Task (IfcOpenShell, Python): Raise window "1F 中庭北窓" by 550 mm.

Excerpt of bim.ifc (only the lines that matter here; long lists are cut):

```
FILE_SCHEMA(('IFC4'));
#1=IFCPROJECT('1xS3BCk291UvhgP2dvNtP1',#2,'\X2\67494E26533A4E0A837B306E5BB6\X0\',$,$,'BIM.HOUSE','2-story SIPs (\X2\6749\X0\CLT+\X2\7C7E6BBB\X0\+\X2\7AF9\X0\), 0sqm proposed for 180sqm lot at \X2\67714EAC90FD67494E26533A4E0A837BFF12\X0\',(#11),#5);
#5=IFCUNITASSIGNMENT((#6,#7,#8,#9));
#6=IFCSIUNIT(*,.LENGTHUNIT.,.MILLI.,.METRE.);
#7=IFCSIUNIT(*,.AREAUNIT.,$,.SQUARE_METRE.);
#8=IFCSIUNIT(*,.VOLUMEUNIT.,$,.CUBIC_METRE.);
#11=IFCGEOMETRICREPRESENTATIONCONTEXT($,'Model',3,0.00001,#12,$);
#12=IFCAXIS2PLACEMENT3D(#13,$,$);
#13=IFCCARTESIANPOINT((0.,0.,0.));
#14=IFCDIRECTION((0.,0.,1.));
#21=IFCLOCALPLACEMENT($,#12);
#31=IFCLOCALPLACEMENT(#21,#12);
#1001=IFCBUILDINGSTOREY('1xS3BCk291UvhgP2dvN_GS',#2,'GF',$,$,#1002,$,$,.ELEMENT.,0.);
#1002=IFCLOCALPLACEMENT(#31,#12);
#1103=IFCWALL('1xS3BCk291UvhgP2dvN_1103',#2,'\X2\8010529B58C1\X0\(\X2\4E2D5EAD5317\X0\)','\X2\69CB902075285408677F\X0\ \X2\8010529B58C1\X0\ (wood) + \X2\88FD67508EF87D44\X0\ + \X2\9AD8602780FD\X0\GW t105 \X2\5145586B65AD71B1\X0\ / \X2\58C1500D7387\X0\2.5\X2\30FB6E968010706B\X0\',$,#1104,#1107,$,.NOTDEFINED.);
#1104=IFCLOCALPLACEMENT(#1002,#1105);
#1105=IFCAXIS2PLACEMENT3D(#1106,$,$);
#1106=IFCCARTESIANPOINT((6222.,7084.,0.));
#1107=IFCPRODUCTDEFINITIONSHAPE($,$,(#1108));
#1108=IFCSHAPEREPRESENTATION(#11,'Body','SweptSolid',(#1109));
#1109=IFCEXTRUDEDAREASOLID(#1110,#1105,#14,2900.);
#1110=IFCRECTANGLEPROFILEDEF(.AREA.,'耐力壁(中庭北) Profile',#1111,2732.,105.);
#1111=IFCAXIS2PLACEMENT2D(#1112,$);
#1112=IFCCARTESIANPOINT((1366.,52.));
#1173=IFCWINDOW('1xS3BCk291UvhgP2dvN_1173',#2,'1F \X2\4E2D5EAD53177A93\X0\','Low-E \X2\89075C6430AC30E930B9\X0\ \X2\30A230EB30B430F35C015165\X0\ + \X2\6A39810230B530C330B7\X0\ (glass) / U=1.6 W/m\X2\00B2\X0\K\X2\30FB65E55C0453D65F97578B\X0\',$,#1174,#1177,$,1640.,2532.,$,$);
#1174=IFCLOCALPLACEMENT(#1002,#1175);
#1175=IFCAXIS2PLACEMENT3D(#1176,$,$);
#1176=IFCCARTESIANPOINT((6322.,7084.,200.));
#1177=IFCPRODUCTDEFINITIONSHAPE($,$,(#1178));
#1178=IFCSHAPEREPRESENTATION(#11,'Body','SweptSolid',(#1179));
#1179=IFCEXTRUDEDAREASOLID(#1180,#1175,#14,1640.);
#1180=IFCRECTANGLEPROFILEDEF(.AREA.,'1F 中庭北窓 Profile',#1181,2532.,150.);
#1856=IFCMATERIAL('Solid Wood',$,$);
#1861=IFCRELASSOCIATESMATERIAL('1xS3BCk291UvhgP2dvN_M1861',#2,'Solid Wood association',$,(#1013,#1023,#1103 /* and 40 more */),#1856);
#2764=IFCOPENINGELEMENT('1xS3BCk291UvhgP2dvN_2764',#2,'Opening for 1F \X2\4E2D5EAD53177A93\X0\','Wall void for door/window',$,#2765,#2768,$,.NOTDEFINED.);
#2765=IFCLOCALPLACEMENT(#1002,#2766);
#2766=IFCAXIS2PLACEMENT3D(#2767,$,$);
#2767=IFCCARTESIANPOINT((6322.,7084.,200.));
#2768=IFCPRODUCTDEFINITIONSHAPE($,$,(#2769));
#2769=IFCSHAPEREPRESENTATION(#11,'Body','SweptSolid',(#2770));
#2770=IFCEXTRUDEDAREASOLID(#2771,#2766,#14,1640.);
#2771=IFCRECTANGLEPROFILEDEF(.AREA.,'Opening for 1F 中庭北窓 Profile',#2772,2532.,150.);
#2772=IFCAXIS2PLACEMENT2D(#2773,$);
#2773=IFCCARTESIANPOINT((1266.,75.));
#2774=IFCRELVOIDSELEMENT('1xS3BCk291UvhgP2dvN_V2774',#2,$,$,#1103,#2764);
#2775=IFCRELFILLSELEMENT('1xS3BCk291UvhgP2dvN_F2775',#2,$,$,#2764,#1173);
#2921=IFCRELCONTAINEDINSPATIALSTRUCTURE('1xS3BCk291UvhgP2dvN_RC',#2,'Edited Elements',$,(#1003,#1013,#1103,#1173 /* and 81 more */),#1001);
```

```python
import numpy as np
import ifcopenshell
import ifcopenshell.api.geometry
import ifcopenshell.util.placement
import ifcopenshell.util.unit

model = ifcopenshell.open("bim.ifc")
unit_scale = ifcopenshell.util.unit.calculate_unit_scale(model)

window = model.by_guid("1xS3BCk291UvhgP2dvN_1173")
opening = window.FillsVoids[0].RelatingOpeningElement
dz = 0.55 / unit_scale

shift = np.array([0.0, 0.0, dz])
# The window is not placed relative to its opening, so move both.
for product in (opening, window):
    matrix = ifcopenshell.util.placement.get_local_placement(product.ObjectPlacement)
    matrix[:3, 3] += shift
    ifcopenshell.api.geometry.edit_object_placement(model, product=product, matrix=matrix, is_si=False)

print(f"moved by {dz * unit_scale:+.3f} m")

model.write("bim_rev.ifc")
```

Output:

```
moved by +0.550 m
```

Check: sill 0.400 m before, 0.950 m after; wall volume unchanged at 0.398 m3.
